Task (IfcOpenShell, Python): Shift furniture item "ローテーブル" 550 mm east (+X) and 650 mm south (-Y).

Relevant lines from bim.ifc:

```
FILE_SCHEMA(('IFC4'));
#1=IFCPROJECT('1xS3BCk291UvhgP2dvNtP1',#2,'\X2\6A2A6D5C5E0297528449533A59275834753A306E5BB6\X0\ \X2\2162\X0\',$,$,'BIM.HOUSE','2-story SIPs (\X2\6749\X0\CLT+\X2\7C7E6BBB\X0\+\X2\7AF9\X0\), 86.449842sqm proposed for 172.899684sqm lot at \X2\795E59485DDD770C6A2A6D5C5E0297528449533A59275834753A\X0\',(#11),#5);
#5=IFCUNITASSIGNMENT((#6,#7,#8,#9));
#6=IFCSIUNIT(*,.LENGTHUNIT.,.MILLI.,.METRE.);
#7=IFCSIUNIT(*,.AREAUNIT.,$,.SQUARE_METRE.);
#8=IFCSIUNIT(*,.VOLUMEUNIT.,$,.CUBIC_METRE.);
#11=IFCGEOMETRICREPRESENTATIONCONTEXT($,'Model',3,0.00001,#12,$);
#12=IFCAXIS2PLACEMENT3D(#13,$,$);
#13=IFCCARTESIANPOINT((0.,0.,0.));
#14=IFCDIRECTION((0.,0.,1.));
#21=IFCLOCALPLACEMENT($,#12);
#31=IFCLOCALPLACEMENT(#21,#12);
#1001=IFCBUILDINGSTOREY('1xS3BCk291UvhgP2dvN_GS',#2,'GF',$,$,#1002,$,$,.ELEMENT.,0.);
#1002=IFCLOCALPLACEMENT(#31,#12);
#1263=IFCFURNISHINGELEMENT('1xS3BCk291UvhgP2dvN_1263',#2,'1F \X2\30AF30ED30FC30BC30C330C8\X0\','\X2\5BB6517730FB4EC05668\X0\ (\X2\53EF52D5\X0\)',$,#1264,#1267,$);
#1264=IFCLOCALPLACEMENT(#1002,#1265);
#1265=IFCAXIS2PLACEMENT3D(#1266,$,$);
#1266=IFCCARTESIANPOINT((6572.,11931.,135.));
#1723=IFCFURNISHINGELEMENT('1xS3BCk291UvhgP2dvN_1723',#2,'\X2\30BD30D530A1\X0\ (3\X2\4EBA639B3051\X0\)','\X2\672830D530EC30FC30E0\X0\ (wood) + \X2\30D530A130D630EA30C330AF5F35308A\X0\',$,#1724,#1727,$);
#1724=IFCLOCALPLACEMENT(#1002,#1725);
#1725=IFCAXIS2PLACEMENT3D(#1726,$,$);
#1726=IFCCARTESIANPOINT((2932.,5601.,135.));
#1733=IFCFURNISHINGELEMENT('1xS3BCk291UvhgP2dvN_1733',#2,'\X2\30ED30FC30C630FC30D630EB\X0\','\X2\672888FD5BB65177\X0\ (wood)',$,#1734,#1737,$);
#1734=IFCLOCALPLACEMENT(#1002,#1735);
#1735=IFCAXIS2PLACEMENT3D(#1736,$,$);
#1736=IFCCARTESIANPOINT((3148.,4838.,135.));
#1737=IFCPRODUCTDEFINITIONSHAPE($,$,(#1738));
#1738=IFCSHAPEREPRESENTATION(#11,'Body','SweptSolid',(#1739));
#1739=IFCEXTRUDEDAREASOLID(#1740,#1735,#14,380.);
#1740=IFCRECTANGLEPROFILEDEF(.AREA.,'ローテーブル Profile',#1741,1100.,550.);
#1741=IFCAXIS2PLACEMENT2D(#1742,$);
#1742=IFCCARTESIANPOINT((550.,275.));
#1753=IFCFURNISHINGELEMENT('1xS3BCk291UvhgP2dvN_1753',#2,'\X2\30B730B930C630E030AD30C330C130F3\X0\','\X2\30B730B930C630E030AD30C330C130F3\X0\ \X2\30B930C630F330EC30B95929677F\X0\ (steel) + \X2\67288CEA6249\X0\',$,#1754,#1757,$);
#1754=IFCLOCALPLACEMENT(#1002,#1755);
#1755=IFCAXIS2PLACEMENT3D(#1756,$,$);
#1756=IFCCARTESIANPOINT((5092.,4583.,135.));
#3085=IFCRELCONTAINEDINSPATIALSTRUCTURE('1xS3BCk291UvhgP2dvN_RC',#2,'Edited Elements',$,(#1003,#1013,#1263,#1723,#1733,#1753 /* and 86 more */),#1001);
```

```python
import ifcopenshell
import ifcopenshell.api.geometry
import ifcopenshell.util.placement
import ifcopenshell.util.unit

model = ifcopenshell.open("bim.ifc")
unit_scale = ifcopenshell.util.unit.calculate_unit_scale(model)

item = model.by_guid("1xS3BCk291UvhgP2dvN_1733")
matrix = ifcopenshell.util.placement.get_local_placement(item.ObjectPlacement)
matrix[0, 3] += 0.55 / unit_scale
matrix[1, 3] -= 0.65 / unit_scale
ifcopenshell.api.geometry.edit_object_placement(model, product=item, matrix=matrix, is_si=False)

print(ifcopenshell.util.placement.get_local_placement(item.ObjectPlacement).round(3) + 0.0)

model.write("bim_v2.ifc")
```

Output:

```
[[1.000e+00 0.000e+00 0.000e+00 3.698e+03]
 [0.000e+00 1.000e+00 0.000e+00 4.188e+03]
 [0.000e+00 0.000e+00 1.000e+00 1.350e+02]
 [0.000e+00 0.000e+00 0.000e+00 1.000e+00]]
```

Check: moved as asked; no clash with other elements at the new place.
